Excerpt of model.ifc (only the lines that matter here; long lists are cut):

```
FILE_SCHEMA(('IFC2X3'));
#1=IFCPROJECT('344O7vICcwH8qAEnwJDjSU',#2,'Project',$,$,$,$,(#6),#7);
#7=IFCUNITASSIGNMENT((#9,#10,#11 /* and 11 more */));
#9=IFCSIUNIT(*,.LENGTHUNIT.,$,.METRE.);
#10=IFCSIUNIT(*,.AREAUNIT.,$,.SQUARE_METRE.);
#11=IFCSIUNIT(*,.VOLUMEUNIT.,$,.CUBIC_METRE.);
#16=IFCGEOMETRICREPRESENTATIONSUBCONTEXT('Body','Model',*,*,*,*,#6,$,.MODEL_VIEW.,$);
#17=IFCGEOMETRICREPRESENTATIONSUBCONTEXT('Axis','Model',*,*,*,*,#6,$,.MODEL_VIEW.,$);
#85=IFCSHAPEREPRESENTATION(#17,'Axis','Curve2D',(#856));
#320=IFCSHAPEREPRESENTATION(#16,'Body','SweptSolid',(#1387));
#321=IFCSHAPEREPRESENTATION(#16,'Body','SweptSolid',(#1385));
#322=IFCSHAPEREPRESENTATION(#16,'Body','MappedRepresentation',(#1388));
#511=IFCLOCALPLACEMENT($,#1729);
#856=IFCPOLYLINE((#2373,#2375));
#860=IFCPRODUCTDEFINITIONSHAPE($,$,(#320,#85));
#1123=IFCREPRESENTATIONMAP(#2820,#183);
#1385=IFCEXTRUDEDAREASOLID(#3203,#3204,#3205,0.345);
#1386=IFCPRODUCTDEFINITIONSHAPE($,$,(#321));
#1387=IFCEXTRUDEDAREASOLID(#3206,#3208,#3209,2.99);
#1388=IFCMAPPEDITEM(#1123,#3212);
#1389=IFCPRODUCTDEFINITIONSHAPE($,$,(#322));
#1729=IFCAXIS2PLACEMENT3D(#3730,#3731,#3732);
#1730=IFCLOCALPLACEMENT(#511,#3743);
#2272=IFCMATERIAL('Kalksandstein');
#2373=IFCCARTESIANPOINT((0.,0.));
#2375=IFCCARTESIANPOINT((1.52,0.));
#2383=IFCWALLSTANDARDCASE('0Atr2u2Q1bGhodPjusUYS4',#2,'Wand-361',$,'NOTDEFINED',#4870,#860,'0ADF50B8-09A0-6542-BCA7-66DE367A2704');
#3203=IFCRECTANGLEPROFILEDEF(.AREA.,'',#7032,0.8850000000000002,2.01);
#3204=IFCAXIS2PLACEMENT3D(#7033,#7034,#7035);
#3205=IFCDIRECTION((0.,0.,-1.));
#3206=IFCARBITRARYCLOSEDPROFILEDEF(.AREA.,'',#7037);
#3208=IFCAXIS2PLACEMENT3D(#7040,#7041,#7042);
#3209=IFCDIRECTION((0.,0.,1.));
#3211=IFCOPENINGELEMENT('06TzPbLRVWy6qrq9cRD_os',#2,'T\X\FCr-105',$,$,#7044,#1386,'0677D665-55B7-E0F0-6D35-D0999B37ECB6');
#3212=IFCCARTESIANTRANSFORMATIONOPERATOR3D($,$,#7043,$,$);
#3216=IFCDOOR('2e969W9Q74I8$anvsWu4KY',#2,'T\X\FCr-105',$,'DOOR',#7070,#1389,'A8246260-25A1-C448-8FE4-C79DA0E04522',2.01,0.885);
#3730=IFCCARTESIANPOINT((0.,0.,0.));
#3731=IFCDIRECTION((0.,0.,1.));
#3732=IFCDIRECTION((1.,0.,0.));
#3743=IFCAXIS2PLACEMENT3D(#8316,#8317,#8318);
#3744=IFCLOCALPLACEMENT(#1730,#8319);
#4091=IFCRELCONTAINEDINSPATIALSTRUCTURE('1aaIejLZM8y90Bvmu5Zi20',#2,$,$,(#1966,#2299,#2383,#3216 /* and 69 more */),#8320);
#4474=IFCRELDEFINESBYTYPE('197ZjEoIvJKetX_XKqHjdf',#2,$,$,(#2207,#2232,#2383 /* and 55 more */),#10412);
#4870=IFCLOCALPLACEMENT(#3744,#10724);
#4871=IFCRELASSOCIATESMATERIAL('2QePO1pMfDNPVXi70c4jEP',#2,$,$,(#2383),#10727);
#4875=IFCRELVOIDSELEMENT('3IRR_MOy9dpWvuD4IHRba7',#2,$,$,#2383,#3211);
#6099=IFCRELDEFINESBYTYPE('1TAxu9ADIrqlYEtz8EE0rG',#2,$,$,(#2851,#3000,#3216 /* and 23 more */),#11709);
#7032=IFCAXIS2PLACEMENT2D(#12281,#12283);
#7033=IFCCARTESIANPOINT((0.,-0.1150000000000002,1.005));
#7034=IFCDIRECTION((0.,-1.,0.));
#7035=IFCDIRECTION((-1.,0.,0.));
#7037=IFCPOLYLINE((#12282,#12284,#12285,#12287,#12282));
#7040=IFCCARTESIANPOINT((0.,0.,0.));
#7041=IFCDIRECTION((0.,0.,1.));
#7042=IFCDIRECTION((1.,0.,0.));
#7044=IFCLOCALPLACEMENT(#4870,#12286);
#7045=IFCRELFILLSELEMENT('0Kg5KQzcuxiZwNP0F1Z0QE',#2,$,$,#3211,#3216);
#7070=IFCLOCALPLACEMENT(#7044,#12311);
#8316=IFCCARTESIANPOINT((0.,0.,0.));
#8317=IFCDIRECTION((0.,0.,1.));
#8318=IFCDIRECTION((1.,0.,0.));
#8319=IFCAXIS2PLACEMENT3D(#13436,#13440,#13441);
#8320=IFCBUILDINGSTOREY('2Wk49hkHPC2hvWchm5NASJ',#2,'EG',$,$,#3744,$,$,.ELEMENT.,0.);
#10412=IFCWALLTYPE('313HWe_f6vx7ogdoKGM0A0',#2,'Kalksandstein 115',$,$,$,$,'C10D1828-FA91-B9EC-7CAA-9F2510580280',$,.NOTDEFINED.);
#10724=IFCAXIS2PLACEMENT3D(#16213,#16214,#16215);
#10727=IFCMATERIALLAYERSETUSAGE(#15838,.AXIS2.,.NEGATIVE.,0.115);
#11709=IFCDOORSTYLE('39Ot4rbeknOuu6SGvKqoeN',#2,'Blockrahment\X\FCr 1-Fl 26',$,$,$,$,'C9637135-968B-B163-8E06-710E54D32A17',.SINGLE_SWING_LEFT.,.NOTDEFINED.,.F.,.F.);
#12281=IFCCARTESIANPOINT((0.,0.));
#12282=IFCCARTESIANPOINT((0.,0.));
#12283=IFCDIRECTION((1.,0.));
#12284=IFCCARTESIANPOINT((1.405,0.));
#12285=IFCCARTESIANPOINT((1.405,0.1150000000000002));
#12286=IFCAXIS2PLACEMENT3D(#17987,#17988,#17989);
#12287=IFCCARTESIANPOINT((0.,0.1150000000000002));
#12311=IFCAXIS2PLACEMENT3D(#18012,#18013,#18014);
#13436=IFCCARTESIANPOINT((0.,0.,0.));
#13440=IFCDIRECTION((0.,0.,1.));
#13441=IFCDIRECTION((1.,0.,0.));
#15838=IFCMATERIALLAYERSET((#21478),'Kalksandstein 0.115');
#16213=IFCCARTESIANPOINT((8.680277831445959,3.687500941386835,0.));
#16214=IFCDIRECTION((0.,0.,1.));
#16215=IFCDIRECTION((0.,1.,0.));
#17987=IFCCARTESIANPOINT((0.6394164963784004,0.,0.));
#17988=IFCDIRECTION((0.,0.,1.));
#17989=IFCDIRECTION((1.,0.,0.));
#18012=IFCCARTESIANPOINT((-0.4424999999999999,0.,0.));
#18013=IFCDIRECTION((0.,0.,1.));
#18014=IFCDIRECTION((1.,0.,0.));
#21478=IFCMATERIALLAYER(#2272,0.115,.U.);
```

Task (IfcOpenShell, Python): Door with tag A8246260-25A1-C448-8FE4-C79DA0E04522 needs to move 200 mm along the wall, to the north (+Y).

```python
import ifcopenshell
import ifcopenshell.api.geometry
import ifcopenshell.util.placement

model = ifcopenshell.open("model.ifc")

door = model.by_guid("2e969W9Q74I8$anvsWu4KY")
opening = door.FillsVoids[0].RelatingOpeningElement
wall = opening.VoidsElements[0].RelatingBuildingElement

wall_matrix = ifcopenshell.util.placement.get_local_placement(wall.ObjectPlacement)
shift = wall_matrix[:3, 0] * 0.2
before = ifcopenshell.util.placement.get_local_placement(door.ObjectPlacement)[:3, 3].copy()

# The door is placed relative to its opening, so it follows when the opening moves.
matrix = ifcopenshell.util.placement.get_local_placement(opening.ObjectPlacement)
matrix[:3, 3] += shift
ifcopenshell.api.geometry.edit_object_placement(
    model, product=opening, matrix=matrix, is_si=False, should_transform_children=True
)

after = ifcopenshell.util.placement.get_local_placement(door.ObjectPlacement)[:3, 3]
print("door moved by", (after - before).round(3) + 0.0)

model.write("model_rev.ifc")
```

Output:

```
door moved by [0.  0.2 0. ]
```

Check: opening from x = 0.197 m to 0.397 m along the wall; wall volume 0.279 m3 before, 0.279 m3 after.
